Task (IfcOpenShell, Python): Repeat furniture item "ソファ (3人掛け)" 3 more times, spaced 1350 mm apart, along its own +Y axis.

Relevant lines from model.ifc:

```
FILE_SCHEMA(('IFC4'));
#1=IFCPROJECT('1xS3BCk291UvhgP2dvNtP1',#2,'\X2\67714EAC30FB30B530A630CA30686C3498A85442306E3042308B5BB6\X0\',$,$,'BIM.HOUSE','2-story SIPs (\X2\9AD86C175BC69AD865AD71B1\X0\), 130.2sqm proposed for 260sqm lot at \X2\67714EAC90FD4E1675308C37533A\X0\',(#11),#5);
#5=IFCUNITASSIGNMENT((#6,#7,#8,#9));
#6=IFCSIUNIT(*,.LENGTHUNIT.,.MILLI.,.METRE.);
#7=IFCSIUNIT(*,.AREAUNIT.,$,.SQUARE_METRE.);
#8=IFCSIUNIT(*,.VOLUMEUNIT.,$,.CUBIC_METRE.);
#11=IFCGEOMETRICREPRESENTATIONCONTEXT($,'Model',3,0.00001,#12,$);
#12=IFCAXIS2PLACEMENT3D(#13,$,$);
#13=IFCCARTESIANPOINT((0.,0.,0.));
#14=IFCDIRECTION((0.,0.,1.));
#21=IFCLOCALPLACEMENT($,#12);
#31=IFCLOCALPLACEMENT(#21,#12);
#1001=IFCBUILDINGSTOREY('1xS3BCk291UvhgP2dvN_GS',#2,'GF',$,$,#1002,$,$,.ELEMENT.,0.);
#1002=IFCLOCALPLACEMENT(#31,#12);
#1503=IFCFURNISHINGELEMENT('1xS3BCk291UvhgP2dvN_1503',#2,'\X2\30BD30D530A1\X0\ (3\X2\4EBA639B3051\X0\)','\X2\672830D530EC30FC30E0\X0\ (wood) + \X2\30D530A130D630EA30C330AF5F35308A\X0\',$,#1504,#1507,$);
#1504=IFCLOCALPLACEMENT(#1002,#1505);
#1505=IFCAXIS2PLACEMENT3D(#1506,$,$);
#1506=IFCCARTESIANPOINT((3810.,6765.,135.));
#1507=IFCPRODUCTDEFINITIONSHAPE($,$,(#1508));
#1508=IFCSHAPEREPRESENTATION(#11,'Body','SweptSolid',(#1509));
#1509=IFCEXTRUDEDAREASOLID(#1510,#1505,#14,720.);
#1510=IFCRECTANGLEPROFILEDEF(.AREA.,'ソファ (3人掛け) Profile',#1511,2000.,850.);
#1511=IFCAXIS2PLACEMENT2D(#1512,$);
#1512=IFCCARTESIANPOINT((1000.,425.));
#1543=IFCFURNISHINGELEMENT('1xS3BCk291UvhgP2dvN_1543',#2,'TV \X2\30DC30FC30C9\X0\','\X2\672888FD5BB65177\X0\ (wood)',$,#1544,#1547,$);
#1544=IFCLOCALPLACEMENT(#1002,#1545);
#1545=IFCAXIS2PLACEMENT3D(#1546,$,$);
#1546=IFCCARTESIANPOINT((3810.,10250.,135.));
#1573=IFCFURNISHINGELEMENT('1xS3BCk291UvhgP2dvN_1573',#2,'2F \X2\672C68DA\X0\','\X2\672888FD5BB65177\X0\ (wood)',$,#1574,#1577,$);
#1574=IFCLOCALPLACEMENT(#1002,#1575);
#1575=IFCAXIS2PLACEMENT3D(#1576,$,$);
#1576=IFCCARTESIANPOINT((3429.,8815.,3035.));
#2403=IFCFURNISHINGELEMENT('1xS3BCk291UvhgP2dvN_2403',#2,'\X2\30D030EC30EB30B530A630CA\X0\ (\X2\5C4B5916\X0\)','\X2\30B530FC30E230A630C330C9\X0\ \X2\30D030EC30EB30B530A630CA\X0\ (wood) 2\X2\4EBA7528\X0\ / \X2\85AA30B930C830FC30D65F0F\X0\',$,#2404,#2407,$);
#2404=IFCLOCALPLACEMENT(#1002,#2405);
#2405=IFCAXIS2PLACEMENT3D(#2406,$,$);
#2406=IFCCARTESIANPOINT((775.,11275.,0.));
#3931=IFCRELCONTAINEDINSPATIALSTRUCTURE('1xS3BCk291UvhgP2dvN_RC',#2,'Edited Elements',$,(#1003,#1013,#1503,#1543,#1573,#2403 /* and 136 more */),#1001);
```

```python
import ifcopenshell
import ifcopenshell.api.geometry
import ifcopenshell.api.root
import ifcopenshell.util.element
import ifcopenshell.util.placement
import ifcopenshell.util.unit

model = ifcopenshell.open("model.ifc")
unit_scale = ifcopenshell.util.unit.calculate_unit_scale(model)


def reuse_history(source, copy):
    """copy_class also copies each property set's owner history, people and application; keep the originals."""
    for rel in copy.IsDefinedBy:
        if rel.is_a("IfcRelDefinesByProperties") and (history := rel.RelatingPropertyDefinition.OwnerHistory):
            rel.RelatingPropertyDefinition.OwnerHistory = source.OwnerHistory
            ifcopenshell.util.element.remove_deep2(model, history)


source = model.by_id(1503)
base = ifcopenshell.util.placement.get_local_placement(source.ObjectPlacement)
step = base[:3, 1] * 1.35 / unit_scale

for i in range(1, 4):
    copy = ifcopenshell.api.root.copy_class(model, product=source)
    copy.Representation = ifcopenshell.util.element.copy_deep(
        model, source.Representation, exclude=["IfcGeometricRepresentationContext", "IfcRepresentationMap"]
    )
    reuse_history(source, copy)
    matrix = base.copy()
    matrix[:3, 3] += i * step
    print("added at", matrix[:3, 3].round(3) + 0.0)
    ifcopenshell.api.geometry.edit_object_placement(model, product=copy, matrix=matrix, is_si=False)

model.write("model_rev.ifc")
```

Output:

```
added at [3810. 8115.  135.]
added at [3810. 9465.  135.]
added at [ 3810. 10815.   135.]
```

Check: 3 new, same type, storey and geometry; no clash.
